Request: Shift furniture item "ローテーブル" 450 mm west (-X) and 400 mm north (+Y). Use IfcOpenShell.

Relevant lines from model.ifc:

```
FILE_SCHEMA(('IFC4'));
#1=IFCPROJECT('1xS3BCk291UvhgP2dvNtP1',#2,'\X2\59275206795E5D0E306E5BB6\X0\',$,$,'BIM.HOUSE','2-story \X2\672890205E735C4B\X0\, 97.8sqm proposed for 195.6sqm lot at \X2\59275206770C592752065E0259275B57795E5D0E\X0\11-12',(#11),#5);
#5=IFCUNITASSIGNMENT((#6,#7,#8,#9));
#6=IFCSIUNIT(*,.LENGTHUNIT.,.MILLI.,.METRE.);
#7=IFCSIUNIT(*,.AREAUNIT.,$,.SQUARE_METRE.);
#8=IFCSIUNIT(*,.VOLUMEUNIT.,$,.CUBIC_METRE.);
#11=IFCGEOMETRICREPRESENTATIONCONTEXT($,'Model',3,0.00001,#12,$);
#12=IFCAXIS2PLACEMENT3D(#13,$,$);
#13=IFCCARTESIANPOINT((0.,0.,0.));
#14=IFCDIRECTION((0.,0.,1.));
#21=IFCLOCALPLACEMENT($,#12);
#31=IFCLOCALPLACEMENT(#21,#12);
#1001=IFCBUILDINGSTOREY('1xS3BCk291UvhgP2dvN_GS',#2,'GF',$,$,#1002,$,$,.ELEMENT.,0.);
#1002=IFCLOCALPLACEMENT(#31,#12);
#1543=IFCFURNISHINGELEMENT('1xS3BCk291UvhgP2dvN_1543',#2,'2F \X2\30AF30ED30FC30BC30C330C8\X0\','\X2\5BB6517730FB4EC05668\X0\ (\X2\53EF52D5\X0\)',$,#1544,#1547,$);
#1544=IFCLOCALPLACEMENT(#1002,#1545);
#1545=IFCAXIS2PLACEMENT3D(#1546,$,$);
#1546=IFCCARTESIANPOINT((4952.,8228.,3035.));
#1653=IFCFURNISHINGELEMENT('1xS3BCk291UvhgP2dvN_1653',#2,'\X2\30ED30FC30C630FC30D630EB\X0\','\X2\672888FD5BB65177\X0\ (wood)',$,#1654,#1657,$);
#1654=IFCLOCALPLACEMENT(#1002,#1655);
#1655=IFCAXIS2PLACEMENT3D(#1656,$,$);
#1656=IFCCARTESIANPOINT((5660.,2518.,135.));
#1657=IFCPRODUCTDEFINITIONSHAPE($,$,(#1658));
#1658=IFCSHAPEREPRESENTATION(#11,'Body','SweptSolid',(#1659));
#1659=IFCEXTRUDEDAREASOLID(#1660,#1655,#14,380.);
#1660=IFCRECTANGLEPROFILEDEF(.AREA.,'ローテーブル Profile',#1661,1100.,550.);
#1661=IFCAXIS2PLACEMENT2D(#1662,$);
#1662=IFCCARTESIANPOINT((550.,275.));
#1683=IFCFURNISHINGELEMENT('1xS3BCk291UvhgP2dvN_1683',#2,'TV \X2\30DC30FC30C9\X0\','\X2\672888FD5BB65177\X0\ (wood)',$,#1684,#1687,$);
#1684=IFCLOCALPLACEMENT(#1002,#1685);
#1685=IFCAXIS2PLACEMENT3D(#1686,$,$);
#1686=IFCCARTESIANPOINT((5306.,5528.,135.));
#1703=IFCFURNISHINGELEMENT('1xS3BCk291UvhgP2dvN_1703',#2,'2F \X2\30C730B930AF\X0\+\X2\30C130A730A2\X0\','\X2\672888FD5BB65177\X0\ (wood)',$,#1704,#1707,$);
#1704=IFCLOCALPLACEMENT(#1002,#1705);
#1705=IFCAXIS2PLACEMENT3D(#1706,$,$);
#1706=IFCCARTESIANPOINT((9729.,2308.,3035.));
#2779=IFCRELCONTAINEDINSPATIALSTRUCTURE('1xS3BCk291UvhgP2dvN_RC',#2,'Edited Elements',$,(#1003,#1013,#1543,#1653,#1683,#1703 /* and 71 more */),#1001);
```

```python
import ifcopenshell
import ifcopenshell.api.geometry
import ifcopenshell.util.placement
import ifcopenshell.util.unit

model = ifcopenshell.open("model.ifc")
unit_scale = ifcopenshell.util.unit.calculate_unit_scale(model)

item = model.by_guid("1xS3BCk291UvhgP2dvN_1653")
matrix = ifcopenshell.util.placement.get_local_placement(item.ObjectPlacement)
matrix[0, 3] -= 0.45 / unit_scale
matrix[1, 3] += 0.4 / unit_scale
ifcopenshell.api.geometry.edit_object_placement(model, product=item, matrix=matrix, is_si=False)

print(ifcopenshell.util.placement.get_local_placement(item.ObjectPlacement).round(3) + 0.0)

model.write("model_edited.ifc")
```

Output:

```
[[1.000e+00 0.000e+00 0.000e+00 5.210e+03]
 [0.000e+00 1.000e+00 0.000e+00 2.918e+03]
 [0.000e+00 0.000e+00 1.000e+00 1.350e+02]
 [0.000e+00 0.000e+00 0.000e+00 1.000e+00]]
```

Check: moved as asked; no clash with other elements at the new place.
